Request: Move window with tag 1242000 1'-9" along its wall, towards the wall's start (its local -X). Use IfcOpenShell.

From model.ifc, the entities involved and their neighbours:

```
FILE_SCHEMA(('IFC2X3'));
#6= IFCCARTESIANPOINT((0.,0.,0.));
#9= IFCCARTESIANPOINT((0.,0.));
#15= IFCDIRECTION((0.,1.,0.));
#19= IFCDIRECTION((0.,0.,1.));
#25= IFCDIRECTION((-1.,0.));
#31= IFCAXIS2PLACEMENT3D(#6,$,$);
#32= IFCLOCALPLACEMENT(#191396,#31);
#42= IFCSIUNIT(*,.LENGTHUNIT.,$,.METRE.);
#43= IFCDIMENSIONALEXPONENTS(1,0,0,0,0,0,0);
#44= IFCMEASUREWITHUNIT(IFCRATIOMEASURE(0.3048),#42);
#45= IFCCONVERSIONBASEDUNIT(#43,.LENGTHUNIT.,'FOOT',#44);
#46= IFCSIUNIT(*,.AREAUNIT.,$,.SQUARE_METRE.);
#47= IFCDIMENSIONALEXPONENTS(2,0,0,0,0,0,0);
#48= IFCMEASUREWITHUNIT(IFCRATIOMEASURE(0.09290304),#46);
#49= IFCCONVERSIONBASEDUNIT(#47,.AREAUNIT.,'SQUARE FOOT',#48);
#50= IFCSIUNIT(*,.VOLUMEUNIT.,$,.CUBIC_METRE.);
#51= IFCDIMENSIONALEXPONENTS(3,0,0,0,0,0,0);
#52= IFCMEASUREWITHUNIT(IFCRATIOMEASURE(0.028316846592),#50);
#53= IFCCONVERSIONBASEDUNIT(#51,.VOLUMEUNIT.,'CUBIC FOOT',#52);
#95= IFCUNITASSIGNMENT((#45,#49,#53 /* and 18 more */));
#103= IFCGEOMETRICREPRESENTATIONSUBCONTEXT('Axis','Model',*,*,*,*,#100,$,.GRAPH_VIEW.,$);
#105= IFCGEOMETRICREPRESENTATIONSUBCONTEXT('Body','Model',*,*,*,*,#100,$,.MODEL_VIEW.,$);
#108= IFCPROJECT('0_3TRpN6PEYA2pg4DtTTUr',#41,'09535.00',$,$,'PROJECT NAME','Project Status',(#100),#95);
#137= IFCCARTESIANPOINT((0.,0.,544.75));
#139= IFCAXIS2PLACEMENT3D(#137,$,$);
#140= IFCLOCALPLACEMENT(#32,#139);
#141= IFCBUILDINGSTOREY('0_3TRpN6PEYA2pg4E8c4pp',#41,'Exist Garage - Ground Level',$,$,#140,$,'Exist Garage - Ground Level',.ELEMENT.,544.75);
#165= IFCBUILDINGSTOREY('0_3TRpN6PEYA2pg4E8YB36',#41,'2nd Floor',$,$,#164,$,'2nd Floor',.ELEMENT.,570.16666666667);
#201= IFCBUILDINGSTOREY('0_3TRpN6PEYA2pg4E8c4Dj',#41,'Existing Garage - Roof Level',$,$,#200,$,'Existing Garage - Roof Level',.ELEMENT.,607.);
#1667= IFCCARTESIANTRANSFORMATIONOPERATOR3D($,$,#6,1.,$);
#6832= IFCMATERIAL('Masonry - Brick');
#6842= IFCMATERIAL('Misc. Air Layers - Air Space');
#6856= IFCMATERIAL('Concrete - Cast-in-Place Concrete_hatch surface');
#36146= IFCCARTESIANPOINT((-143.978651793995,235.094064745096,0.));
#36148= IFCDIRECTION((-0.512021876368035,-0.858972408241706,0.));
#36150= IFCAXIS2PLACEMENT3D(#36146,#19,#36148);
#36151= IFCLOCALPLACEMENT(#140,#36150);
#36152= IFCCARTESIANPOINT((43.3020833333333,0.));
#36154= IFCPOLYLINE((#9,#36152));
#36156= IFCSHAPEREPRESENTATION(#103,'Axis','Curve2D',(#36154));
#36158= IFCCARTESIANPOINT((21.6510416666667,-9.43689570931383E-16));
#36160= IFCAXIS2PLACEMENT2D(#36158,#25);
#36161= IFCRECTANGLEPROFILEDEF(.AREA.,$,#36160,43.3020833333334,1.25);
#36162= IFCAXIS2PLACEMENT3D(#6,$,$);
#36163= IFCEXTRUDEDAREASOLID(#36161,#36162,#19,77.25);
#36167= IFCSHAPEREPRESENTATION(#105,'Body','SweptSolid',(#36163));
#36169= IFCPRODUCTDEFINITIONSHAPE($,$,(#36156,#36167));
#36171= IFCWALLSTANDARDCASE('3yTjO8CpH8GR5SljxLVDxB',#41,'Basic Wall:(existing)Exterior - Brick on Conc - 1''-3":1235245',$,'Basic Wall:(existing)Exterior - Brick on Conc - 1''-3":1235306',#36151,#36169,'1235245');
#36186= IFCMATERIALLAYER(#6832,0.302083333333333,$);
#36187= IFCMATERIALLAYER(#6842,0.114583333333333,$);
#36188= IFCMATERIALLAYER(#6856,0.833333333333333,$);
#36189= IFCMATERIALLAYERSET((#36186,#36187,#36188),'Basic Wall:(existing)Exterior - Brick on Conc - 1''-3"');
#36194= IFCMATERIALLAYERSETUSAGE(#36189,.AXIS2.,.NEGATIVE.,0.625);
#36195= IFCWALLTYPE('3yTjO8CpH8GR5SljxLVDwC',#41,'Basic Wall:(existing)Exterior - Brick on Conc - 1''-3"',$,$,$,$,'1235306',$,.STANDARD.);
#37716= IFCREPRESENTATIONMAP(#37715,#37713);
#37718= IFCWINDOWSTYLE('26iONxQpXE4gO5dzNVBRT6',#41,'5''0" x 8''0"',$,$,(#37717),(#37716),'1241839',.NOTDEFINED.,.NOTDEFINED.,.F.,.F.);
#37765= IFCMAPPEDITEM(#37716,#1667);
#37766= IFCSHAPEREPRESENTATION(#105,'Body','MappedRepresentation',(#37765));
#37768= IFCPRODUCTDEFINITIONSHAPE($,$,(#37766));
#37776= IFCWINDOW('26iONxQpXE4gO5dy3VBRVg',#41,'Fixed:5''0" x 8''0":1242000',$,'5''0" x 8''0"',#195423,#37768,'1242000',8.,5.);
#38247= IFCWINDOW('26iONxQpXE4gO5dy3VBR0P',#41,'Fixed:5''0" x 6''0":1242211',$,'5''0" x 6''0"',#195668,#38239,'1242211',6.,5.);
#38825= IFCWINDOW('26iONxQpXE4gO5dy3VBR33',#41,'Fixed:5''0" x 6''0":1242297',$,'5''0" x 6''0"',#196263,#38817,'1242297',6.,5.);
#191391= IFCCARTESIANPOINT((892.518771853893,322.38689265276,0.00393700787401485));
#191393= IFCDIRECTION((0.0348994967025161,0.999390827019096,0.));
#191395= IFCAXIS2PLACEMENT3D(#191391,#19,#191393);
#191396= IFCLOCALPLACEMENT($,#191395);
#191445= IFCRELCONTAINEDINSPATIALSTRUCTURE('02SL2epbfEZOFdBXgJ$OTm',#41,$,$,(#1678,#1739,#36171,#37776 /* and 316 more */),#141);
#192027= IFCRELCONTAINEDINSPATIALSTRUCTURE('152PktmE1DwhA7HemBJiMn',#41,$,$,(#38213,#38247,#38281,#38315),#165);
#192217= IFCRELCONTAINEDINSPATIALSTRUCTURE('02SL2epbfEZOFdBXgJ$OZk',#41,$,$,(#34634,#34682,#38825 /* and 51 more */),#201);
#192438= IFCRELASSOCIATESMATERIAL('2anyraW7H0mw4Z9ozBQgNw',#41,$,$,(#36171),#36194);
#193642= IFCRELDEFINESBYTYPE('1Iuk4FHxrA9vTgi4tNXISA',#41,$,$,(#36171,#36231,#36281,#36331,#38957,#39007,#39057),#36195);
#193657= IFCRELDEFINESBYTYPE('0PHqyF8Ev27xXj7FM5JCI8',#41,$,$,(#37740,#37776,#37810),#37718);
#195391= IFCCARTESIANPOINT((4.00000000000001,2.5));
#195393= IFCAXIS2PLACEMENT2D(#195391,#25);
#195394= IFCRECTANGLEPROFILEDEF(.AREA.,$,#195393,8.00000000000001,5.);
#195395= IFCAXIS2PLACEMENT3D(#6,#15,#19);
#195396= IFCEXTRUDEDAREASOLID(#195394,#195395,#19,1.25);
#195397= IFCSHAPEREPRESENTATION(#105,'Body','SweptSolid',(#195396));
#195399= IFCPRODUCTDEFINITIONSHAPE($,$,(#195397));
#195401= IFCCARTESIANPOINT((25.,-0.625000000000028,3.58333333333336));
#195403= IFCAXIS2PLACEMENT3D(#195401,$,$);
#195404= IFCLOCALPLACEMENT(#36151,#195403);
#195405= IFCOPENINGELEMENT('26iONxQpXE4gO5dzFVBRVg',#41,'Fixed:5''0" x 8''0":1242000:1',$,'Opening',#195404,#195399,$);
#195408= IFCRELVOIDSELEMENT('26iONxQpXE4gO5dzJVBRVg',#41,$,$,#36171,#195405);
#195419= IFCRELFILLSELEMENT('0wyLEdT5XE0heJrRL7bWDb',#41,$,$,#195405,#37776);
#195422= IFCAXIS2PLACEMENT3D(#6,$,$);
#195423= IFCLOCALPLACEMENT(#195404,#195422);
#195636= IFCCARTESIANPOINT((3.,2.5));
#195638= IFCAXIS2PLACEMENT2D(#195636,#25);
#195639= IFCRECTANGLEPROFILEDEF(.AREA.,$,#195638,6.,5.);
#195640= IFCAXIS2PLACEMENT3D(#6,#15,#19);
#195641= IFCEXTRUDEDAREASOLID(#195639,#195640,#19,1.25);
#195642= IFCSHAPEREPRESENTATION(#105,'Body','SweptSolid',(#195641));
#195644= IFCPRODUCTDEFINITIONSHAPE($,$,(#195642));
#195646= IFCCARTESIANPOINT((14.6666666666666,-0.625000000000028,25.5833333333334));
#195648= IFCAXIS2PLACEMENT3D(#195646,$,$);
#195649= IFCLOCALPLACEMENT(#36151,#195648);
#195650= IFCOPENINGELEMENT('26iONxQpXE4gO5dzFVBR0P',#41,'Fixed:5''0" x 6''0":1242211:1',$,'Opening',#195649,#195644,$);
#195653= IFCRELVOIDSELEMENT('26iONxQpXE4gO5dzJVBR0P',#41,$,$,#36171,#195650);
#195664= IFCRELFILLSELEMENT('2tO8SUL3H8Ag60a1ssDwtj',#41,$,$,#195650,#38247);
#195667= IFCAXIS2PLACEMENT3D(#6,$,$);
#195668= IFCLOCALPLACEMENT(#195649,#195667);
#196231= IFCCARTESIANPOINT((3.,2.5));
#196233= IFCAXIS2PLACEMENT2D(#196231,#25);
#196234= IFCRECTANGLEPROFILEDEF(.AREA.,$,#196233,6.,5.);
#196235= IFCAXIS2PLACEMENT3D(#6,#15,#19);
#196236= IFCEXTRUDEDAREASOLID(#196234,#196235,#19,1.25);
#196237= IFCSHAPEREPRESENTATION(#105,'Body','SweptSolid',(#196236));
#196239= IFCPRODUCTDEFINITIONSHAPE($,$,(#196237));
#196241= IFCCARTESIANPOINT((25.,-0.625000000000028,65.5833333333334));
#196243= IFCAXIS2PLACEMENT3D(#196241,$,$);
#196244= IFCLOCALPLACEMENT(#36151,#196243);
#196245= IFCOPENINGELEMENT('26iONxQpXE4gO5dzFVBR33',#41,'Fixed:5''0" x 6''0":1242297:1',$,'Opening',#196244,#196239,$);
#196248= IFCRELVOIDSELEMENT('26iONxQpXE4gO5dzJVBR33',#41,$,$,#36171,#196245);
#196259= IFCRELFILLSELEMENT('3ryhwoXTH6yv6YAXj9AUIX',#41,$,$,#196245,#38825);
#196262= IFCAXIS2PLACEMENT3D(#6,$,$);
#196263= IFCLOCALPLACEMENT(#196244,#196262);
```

```python
import ifcopenshell
import ifcopenshell.api.geometry
import ifcopenshell.util.placement
import ifcopenshell.util.unit

model = ifcopenshell.open("model.ifc")
unit_scale = ifcopenshell.util.unit.calculate_unit_scale(model)

window = model.by_guid("26iONxQpXE4gO5dy3VBRVg")
opening = window.FillsVoids[0].RelatingOpeningElement
wall = opening.VoidsElements[0].RelatingBuildingElement

wall_matrix = ifcopenshell.util.placement.get_local_placement(wall.ObjectPlacement)
shift = wall_matrix[:3, 0] * -21 * 0.0254 / unit_scale
before = ifcopenshell.util.placement.get_local_placement(window.ObjectPlacement)[:3, 3].copy()

# The window is placed relative to its opening, so it follows when the opening moves.
matrix = ifcopenshell.util.placement.get_local_placement(opening.ObjectPlacement)
matrix[:3, 3] += shift
ifcopenshell.api.geometry.edit_object_placement(
    model, product=opening, matrix=matrix, is_si=False, should_transform_children=True
)

after = ifcopenshell.util.placement.get_local_placement(window.ObjectPlacement)[:3, 3]
print("window moved by", (after - before).round(3) + 0.0)

model.write("model_updated.ifc")
```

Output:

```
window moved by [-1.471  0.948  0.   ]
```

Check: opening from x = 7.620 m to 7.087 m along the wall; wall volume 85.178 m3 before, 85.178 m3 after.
